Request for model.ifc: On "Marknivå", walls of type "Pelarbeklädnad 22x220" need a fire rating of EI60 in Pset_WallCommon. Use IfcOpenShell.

First a look at what the model holds.

```python
import ifcopenshell
import ifcopenshell.util.element

model = ifcopenshell.open("model.ifc")
print(model.schema)
storey = next(s for s in model.by_type("IfcBuildingStorey") if s.Name == "Marknivå")
walls = [e for e in ifcopenshell.util.element.get_decomposition(storey) if e.is_a("IfcWall")]
seen = {}
for e in walls:
    element_type = ifcopenshell.util.element.get_type(e)
    key = (element_type.Name if element_type != e and element_type else None, ifcopenshell.util.element.get_pset(e, "Pset_WallCommon", "FireRating"))
    seen[key] = seen.get(key, 0) + 1
for (name, value), count in sorted(seen.items(), key=str):
    print(count, "x", name, "|", value)
```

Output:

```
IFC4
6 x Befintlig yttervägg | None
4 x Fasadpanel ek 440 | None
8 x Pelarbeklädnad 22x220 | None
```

```python
import ifcopenshell
import ifcopenshell.api.pset
import ifcopenshell.util.element

model = ifcopenshell.open("model.ifc")

storey = next(s for s in model.by_type("IfcBuildingStorey") if s.Name == "Marknivå")
walls = [e for e in ifcopenshell.util.element.get_decomposition(storey) if e.is_a("IfcWall")]

count = 0
for e in walls:
    element_type = ifcopenshell.util.element.get_type(e)
    if element_type in (None, e) or element_type.Name != "Pelarbeklädnad 22x220":
        continue
    # add_pset returns the element's existing set when there is one.
    pset = ifcopenshell.api.pset.add_pset(model, product=e, name="Pset_WallCommon")
    ifcopenshell.api.pset.edit_pset(model, pset=pset, properties={"FireRating": "EI60"})
    count += 1

print(count, "walls updated")

model.write("model_v2.ifc")
```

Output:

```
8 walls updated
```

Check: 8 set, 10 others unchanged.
